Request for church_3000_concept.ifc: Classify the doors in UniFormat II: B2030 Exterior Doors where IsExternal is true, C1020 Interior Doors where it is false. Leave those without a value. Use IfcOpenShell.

First a look at what the model holds.

```python
import ifcopenshell
import ifcopenshell.util.element

model = ifcopenshell.open("church_3000_concept.ifc")
print(model.schema)
print("classifications:", [c.Name for c in model.by_type("IfcClassification")])
values = [ifcopenshell.util.element.get_pset(e, "Pset_DoorCommon", "IsExternal") for e in model.by_type("IfcDoor")]
for value in (True, False, None):
    print("IsExternal", value, values.count(value))
```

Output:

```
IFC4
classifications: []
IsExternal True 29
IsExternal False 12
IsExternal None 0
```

```python
import ifcopenshell
import ifcopenshell.api.classification
import ifcopenshell.util.element

model = ifcopenshell.open("church_3000_concept.ifc")

system = ifcopenshell.api.classification.add_classification(model, classification="UniFormat II")

doors = model.by_type("IfcDoor")
external = {e: ifcopenshell.util.element.get_pset(e, "Pset_DoorCommon", "IsExternal") for e in doors}
for flag, code, name in ((True, "B2030", "Exterior Doors"), (False, "C1020", "Interior Doors")):
    products = [e for e in doors if external[e] is flag]
    ifcopenshell.api.classification.add_reference(
        model, products=products, classification=system, identification=code, name=name
    )
    print(code, len(products))

model.write("church_3000_concept_rev.ifc")
```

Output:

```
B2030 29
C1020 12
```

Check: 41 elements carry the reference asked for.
